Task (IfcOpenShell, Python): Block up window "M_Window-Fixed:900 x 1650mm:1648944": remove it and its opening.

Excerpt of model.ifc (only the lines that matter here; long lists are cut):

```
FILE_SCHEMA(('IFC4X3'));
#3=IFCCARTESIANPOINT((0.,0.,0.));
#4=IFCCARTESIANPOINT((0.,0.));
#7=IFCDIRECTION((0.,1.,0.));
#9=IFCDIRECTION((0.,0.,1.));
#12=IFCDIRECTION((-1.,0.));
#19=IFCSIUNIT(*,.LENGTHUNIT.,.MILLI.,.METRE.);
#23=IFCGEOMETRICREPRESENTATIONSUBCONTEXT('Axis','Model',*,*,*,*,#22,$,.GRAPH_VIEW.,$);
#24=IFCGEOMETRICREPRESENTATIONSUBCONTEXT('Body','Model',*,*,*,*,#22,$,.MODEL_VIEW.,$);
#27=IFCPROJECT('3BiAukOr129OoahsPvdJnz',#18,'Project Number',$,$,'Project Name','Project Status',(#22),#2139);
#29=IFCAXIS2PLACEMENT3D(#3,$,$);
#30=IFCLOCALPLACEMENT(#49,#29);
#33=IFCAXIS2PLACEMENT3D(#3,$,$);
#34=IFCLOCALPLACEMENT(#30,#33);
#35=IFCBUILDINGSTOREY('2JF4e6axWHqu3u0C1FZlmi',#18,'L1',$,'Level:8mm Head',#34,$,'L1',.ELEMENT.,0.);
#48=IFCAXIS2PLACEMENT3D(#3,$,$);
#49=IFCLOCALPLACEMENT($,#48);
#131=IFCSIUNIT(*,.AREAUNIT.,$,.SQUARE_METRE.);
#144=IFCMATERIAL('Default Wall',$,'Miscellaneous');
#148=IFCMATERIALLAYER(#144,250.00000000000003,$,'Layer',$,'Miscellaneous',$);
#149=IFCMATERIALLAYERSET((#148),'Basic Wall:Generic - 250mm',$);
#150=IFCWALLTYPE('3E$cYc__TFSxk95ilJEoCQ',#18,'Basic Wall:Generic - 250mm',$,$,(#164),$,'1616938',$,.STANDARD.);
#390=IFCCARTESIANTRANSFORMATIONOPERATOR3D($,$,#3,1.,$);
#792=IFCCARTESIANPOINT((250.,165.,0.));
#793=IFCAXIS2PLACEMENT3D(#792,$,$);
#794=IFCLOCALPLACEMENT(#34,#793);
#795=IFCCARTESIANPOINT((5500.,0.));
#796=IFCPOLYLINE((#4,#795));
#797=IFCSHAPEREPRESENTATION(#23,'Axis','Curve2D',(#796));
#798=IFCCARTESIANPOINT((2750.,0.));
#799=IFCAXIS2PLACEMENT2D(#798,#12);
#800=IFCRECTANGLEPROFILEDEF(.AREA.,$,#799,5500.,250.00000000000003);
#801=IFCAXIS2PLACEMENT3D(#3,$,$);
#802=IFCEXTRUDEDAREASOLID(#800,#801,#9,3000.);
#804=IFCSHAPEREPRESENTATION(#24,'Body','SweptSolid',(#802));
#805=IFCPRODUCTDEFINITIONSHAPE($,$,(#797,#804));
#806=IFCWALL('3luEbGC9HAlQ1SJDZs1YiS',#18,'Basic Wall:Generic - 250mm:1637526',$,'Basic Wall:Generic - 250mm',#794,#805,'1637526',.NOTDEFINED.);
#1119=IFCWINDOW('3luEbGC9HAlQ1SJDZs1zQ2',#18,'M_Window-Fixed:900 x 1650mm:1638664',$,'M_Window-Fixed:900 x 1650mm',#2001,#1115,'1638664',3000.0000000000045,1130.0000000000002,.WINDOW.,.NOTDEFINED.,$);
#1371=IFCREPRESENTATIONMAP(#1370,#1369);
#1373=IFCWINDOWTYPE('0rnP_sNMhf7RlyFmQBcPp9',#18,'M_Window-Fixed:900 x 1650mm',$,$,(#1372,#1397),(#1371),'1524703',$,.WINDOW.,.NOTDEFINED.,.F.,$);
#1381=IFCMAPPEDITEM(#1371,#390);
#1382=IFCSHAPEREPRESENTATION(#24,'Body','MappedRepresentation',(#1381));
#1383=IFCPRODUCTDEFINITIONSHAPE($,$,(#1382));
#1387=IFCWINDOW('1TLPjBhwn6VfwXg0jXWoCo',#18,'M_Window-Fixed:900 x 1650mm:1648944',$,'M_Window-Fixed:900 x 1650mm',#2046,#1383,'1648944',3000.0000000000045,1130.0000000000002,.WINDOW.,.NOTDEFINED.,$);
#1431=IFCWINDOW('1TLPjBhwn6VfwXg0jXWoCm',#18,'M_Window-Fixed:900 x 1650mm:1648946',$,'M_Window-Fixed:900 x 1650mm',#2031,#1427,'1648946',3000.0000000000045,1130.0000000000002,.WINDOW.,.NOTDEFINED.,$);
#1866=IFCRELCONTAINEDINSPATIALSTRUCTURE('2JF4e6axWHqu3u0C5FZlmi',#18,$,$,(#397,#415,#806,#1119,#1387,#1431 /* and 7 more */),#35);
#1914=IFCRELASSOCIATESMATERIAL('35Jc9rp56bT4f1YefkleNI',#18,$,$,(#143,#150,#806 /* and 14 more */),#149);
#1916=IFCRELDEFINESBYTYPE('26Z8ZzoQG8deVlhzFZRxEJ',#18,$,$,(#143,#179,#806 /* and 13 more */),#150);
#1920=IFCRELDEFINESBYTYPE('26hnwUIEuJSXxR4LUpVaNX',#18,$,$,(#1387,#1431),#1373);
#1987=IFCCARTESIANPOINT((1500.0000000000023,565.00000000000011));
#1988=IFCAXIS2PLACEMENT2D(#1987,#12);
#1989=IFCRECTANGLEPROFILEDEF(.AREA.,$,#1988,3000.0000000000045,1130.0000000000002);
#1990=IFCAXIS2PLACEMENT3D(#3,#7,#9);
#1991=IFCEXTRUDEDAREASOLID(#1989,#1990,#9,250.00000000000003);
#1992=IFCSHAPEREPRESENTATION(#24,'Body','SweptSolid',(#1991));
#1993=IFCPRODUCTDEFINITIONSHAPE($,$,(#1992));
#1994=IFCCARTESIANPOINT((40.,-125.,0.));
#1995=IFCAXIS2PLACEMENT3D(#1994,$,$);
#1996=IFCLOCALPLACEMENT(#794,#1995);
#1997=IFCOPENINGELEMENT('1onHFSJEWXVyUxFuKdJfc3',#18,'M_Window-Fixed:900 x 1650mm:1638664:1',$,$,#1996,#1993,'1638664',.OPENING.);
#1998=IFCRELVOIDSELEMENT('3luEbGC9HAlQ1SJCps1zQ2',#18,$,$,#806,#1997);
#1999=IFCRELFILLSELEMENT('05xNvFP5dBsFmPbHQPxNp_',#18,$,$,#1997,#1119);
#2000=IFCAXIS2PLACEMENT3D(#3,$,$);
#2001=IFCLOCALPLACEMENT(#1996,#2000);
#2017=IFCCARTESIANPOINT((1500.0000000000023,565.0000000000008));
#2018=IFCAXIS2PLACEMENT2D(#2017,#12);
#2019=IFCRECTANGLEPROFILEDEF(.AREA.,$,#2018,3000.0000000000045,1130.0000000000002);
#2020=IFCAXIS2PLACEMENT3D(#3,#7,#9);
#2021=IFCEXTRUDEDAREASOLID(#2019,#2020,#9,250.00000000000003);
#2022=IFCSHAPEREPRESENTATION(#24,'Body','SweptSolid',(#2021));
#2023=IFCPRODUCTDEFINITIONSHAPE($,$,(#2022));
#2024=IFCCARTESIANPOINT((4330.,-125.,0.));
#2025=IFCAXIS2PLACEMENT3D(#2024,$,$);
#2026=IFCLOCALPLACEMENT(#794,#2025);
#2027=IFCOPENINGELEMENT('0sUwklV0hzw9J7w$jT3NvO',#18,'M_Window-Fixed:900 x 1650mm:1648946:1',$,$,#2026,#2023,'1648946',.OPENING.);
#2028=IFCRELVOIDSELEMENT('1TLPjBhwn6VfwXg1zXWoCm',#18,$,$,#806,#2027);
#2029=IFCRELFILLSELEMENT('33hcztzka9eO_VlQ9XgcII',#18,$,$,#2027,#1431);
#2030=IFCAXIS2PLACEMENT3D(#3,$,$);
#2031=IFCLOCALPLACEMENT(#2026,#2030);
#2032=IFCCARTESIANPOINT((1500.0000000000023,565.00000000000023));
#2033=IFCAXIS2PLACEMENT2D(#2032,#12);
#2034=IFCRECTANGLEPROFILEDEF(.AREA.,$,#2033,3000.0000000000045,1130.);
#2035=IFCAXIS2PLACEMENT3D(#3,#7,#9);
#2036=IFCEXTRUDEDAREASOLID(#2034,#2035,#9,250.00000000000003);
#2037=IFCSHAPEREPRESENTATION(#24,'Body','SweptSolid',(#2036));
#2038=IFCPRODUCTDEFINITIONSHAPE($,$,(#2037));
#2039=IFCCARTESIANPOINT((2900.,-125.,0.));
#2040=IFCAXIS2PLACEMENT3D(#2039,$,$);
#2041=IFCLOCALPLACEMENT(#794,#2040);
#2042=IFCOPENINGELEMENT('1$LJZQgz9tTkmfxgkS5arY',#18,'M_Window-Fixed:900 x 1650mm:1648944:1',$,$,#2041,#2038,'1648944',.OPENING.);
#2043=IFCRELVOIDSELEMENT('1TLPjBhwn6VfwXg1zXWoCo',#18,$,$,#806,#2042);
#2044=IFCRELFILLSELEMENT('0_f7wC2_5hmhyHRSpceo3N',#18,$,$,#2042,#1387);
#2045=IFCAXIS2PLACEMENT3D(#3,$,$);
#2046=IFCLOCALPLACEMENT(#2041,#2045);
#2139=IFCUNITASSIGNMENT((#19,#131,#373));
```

```python
import ifcopenshell
import ifcopenshell.api.feature
import ifcopenshell.api.root
import ifcopenshell.geom
import ifcopenshell.util.shape

model = ifcopenshell.open("model.ifc")
settings = ifcopenshell.geom.settings()


def volume(element):
    """Net volume in cubic metres, openings subtracted."""
    shape = ifcopenshell.geom.create_shape(settings, element)
    return ifcopenshell.util.shape.get_volume(shape.geometry)


window = model.by_guid("1TLPjBhwn6VfwXg0jXWoCo")
opening = window.FillsVoids[0].RelatingOpeningElement
wall = opening.VoidsElements[0].RelatingBuildingElement
before = volume(wall)

ifcopenshell.api.root.remove_product(model, product=window)
ifcopenshell.api.feature.remove_feature(model, feature=opening)

after = volume(wall)

print(f"wall volume {before:.3f} -> {after:.3f} m3")

model.write("model-out.ifc")
```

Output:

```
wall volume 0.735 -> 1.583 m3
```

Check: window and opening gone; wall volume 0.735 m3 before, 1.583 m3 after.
